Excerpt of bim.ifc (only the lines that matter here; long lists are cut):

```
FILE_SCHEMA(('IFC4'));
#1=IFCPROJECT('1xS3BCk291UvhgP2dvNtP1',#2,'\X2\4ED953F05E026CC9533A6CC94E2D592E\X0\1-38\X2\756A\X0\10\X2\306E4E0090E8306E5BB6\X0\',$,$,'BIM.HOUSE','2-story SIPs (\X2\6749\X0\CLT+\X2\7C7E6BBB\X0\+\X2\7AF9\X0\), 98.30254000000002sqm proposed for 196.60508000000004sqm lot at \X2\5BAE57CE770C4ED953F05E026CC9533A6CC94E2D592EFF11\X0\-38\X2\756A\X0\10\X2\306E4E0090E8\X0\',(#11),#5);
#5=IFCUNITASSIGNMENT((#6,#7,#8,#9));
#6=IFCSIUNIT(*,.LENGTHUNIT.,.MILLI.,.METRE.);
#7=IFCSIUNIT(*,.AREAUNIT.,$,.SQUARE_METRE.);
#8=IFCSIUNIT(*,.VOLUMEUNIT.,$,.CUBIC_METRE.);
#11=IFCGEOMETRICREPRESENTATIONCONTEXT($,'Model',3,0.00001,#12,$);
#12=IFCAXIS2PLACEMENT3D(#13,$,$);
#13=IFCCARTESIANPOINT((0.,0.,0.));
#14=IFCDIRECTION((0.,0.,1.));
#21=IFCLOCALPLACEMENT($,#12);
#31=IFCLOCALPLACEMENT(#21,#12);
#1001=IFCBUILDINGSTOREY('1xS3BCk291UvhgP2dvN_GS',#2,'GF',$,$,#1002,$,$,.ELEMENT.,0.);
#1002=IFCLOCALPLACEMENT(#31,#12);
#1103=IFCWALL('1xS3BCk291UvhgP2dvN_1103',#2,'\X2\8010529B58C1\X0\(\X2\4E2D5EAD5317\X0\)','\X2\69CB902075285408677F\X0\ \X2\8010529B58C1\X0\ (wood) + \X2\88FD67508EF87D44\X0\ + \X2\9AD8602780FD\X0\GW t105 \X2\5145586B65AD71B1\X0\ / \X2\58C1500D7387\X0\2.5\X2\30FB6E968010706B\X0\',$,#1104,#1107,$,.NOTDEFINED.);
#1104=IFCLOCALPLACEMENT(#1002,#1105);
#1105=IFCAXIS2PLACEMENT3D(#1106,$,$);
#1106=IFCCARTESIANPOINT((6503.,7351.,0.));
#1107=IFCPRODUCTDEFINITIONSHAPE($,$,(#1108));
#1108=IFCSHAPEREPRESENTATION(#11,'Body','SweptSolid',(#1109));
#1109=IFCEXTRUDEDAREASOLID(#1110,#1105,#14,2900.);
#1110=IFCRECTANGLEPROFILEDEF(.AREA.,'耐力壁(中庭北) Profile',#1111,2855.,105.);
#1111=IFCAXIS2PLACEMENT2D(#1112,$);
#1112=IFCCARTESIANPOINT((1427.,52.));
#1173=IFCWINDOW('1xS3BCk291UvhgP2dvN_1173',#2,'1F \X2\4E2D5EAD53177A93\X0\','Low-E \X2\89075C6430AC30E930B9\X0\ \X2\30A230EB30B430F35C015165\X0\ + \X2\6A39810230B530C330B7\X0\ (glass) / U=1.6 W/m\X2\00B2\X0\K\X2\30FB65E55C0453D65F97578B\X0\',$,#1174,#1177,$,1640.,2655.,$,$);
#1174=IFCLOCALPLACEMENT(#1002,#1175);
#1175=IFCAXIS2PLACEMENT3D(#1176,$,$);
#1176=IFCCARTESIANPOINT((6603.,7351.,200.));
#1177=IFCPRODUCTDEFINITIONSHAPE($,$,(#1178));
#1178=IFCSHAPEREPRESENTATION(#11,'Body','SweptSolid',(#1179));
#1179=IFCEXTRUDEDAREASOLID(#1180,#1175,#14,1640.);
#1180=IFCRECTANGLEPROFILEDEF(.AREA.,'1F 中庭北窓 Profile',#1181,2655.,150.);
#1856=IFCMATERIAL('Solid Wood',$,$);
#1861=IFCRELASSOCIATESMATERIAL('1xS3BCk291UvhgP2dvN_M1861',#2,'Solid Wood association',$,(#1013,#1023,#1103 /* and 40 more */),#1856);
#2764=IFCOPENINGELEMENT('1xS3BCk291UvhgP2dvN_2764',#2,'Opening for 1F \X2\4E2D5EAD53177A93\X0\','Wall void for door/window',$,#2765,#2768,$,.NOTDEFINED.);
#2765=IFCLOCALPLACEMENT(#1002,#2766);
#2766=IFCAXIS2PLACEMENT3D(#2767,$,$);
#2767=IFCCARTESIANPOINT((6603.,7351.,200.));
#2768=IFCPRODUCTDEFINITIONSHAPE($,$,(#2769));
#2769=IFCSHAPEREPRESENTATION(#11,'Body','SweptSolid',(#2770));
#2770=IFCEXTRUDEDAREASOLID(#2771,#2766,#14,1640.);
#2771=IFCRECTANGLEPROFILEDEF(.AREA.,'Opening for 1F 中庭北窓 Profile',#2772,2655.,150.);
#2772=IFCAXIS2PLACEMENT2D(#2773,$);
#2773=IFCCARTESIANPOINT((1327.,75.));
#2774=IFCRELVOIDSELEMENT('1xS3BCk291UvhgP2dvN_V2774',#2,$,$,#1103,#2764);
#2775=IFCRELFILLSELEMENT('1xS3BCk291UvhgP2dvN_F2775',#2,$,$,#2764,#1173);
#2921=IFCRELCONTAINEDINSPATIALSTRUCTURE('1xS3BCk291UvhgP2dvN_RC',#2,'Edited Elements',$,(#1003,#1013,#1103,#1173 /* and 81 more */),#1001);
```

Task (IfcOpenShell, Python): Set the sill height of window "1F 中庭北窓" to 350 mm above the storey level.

```python
import numpy as np
import ifcopenshell
import ifcopenshell.api.geometry
import ifcopenshell.geom
import ifcopenshell.util.element
import ifcopenshell.util.placement
import ifcopenshell.util.shape
import ifcopenshell.util.unit

model = ifcopenshell.open("bim.ifc")
unit_scale = ifcopenshell.util.unit.calculate_unit_scale(model)

window = model.by_guid("1xS3BCk291UvhgP2dvN_1173")
opening = window.FillsVoids[0].RelatingOpeningElement
storey = ifcopenshell.util.element.get_container(window, ifc_class="IfcBuildingStorey")
level = ifcopenshell.util.placement.get_local_placement(storey.ObjectPlacement)[2, 3]

# The opening's origin need not be at the sill, so measure its lowest point.
shape = ifcopenshell.geom.create_shape(ifcopenshell.geom.settings(), opening)
bottom = ifcopenshell.util.shape.get_shape_bottom_elevation(shape, shape.geometry) / unit_scale
dz = level + 0.35 / unit_scale - bottom

shift = np.array([0.0, 0.0, dz])
# The window is not placed relative to its opening, so move both.
for product in (opening, window):
    matrix = ifcopenshell.util.placement.get_local_placement(product.ObjectPlacement)
    matrix[:3, 3] += shift
    ifcopenshell.api.geometry.edit_object_placement(model, product=product, matrix=matrix, is_si=False)

print(f"moved by {dz * unit_scale:+.3f} m")

model.write("bim-out.ifc")
```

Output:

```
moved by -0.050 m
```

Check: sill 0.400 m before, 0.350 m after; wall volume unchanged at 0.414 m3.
